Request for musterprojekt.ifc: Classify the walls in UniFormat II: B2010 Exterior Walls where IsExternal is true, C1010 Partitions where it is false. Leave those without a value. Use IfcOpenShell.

First a look at what the model holds.

```python
import ifcopenshell
import ifcopenshell.util.element

model = ifcopenshell.open("musterprojekt.ifc")
print(model.schema)
print("classifications:", [c.Name for c in model.by_type("IfcClassification")])
values = [ifcopenshell.util.element.get_pset(e, "Pset_WallCommon", "IsExternal") for e in model.by_type("IfcWall")]
for value in (True, False, None):
    print("IsExternal", value, values.count(value))
```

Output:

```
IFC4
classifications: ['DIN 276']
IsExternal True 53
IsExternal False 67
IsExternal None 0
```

```python
import ifcopenshell
import ifcopenshell.api.classification
import ifcopenshell.util.element

model = ifcopenshell.open("musterprojekt.ifc")

system = ifcopenshell.api.classification.add_classification(model, classification="UniFormat II")

walls = model.by_type("IfcWall")
external = {e: ifcopenshell.util.element.get_pset(e, "Pset_WallCommon", "IsExternal") for e in walls}
for flag, code, name in ((True, "B2010", "Exterior Walls"), (False, "C1010", "Partitions")):
    products = [e for e in walls if external[e] is flag]
    ifcopenshell.api.classification.add_reference(
        model, products=products, classification=system, identification=code, name=name
    )
    print(code, len(products))

model.write("musterprojekt-out.ifc")
```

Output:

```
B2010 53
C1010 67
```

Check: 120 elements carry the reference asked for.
